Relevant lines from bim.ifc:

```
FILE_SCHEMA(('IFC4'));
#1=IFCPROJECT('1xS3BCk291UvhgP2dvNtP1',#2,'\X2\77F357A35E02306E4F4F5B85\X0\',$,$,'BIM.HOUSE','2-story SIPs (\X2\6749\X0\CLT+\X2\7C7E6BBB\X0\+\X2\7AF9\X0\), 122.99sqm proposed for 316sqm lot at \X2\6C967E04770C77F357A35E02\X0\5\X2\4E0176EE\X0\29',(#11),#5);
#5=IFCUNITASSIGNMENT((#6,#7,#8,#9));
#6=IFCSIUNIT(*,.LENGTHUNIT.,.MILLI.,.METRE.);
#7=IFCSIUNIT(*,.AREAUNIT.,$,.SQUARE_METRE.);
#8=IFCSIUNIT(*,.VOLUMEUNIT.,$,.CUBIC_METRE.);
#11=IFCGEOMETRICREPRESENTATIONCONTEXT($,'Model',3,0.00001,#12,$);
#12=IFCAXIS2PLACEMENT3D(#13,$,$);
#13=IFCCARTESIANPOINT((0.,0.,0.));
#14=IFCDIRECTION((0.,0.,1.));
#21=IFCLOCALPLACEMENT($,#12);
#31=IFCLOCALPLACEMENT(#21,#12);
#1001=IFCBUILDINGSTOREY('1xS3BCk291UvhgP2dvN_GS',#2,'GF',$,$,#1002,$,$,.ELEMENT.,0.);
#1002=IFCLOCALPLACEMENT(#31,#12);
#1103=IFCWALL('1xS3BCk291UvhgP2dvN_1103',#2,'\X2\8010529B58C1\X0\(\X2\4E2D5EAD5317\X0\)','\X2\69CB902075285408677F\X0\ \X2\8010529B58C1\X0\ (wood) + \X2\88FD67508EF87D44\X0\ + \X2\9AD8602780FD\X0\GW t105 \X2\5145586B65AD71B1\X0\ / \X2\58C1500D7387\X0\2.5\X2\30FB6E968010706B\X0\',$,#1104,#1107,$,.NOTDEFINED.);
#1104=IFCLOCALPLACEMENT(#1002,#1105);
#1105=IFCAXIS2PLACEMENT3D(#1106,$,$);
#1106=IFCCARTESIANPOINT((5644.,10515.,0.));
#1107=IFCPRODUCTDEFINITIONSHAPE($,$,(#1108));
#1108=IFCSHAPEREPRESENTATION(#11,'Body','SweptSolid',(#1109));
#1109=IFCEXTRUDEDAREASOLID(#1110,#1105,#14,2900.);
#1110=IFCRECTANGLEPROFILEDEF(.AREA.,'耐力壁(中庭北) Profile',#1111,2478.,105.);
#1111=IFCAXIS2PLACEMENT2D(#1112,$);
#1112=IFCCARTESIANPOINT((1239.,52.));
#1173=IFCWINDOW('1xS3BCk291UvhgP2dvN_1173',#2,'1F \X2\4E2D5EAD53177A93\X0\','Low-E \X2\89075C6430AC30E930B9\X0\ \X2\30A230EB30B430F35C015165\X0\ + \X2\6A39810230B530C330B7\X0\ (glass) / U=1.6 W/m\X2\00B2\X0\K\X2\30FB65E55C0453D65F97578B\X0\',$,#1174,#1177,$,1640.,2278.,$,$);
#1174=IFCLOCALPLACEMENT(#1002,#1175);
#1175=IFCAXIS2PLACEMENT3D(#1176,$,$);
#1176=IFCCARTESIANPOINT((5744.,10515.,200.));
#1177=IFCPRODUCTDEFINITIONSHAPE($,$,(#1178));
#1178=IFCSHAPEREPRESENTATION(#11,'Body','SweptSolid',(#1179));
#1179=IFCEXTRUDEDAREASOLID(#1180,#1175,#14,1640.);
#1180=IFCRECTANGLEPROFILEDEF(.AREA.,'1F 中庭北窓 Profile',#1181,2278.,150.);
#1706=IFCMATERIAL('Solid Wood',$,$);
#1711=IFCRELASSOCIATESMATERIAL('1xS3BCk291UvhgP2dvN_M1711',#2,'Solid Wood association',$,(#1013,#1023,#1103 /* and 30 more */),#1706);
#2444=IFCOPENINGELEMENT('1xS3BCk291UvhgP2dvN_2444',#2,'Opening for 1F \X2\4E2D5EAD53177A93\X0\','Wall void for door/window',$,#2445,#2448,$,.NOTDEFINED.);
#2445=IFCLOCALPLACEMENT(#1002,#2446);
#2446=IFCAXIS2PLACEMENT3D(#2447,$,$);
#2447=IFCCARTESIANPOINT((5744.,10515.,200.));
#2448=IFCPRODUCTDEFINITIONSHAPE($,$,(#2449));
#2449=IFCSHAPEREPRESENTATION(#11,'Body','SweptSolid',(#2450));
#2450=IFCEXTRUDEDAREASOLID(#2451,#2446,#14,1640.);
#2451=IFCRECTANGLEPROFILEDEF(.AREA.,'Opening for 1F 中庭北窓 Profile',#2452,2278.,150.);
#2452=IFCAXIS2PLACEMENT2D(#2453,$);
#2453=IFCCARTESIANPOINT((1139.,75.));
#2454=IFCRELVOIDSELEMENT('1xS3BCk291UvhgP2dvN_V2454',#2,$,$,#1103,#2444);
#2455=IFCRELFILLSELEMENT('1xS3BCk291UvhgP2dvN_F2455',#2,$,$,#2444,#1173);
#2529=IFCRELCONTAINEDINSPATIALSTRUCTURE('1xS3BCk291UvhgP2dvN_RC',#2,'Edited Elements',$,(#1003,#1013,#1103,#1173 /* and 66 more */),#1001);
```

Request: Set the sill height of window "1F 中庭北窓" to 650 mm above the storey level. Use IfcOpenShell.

```python
import numpy as np
import ifcopenshell
import ifcopenshell.api.geometry
import ifcopenshell.geom
import ifcopenshell.util.element
import ifcopenshell.util.placement
import ifcopenshell.util.shape
import ifcopenshell.util.unit

model = ifcopenshell.open("bim.ifc")
unit_scale = ifcopenshell.util.unit.calculate_unit_scale(model)

window = model.by_id(1173)
opening = window.FillsVoids[0].RelatingOpeningElement
storey = ifcopenshell.util.element.get_container(window, ifc_class="IfcBuildingStorey")
level = ifcopenshell.util.placement.get_local_placement(storey.ObjectPlacement)[2, 3]

# The opening's origin need not be at the sill, so measure its lowest point.
shape = ifcopenshell.geom.create_shape(ifcopenshell.geom.settings(), opening)
bottom = ifcopenshell.util.shape.get_shape_bottom_elevation(shape, shape.geometry) / unit_scale
dz = level + 0.65 / unit_scale - bottom

shift = np.array([0.0, 0.0, dz])
# The window is not placed relative to its opening, so move both.
for product in (opening, window):
    matrix = ifcopenshell.util.placement.get_local_placement(product.ObjectPlacement)
    matrix[:3, 3] += shift
    ifcopenshell.api.geometry.edit_object_placement(model, product=product, matrix=matrix, is_si=False)

print(f"moved by {dz * unit_scale:+.3f} m")

model.write("bim_rev.ifc")
```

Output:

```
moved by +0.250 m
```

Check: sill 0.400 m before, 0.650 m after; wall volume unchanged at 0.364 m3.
